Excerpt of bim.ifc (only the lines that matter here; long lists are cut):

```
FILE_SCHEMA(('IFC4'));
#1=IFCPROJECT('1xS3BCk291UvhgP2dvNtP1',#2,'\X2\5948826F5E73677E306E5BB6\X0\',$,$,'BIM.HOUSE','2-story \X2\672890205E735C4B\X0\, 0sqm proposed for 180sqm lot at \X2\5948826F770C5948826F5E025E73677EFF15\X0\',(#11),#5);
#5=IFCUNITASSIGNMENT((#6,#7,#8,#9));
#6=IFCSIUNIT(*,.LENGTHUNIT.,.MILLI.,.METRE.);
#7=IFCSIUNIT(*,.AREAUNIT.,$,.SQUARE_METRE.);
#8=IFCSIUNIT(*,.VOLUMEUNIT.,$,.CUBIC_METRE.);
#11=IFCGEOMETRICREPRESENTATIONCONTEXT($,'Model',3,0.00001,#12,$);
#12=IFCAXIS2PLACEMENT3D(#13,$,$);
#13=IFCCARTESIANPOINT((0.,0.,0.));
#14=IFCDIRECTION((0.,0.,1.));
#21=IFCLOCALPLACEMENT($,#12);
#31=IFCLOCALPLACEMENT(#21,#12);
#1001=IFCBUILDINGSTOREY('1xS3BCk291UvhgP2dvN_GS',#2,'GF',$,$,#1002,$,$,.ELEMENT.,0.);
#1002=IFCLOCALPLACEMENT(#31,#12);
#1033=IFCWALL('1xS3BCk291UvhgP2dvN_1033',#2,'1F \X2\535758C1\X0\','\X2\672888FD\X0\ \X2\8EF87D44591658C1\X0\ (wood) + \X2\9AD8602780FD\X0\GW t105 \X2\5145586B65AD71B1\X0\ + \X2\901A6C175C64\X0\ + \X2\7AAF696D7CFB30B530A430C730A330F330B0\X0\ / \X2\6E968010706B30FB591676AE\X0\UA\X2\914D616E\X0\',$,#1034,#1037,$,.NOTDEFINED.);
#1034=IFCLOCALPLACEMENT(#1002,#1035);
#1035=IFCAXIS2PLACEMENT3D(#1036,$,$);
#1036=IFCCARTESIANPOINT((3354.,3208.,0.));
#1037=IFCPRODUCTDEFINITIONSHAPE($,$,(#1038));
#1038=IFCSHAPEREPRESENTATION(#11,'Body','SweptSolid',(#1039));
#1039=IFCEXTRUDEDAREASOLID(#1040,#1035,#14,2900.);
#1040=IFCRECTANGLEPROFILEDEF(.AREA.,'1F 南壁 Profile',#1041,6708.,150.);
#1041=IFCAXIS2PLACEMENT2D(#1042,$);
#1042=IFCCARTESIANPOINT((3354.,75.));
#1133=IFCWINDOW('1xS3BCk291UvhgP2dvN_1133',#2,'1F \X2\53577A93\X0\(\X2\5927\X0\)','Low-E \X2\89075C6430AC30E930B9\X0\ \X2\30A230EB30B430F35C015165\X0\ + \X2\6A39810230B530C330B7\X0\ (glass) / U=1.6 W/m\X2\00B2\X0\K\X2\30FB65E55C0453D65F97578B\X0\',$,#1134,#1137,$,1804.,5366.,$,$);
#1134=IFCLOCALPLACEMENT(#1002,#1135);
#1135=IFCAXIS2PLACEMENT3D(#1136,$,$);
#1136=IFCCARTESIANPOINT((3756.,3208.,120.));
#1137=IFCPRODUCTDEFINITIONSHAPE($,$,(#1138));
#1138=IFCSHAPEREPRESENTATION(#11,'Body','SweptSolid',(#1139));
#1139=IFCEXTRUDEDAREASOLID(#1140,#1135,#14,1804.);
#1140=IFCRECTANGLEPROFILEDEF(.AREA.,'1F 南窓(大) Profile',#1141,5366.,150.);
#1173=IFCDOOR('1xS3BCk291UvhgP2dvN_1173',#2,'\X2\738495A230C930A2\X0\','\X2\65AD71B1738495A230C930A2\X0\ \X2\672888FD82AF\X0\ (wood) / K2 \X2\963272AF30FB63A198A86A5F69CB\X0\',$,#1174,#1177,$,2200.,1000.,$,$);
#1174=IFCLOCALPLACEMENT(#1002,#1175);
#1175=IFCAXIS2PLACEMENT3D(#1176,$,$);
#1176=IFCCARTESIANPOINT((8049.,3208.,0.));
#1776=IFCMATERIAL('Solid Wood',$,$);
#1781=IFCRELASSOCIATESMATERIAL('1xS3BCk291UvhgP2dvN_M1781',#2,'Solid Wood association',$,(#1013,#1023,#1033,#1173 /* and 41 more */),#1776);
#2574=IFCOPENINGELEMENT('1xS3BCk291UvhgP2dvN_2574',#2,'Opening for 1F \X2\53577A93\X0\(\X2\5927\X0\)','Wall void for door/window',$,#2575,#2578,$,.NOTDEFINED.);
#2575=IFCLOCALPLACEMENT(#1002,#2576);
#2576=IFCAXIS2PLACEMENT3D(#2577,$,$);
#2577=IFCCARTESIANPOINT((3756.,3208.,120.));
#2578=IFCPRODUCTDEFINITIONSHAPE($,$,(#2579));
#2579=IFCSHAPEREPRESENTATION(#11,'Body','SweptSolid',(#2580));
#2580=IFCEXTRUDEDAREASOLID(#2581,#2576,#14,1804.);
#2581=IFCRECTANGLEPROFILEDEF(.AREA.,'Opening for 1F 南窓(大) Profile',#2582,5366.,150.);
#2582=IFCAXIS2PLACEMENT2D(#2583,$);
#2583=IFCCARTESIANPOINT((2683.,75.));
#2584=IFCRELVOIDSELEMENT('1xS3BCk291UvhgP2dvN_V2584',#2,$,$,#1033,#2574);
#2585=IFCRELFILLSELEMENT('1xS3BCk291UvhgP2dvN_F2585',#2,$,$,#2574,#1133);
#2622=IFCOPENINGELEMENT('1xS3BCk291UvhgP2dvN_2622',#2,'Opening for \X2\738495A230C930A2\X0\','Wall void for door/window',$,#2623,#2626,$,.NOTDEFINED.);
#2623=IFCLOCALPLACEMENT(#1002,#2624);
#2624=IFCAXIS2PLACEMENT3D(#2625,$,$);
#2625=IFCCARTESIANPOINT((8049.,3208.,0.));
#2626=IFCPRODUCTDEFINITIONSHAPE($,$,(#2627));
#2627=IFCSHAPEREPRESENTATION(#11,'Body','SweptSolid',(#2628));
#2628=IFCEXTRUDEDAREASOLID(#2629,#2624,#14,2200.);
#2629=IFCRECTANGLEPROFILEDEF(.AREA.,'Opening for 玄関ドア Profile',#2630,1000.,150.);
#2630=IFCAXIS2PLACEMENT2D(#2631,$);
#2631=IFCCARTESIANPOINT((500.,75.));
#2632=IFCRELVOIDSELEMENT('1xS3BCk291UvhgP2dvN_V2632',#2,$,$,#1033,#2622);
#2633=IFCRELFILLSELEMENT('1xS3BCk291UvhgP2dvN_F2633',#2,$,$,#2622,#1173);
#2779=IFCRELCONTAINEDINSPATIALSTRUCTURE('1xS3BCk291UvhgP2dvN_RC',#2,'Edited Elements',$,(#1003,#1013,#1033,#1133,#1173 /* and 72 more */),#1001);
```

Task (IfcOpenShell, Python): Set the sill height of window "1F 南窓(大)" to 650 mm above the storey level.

```python
import numpy as np
import ifcopenshell
import ifcopenshell.api.geometry
import ifcopenshell.geom
import ifcopenshell.util.element
import ifcopenshell.util.placement
import ifcopenshell.util.shape
import ifcopenshell.util.unit

model = ifcopenshell.open("bim.ifc")
unit_scale = ifcopenshell.util.unit.calculate_unit_scale(model)

window = model.by_guid("1xS3BCk291UvhgP2dvN_1133")
opening = window.FillsVoids[0].RelatingOpeningElement
storey = ifcopenshell.util.element.get_container(window, ifc_class="IfcBuildingStorey")
level = ifcopenshell.util.placement.get_local_placement(storey.ObjectPlacement)[2, 3]

# The opening's origin need not be at the sill, so measure its lowest point.
shape = ifcopenshell.geom.create_shape(ifcopenshell.geom.settings(), opening)
bottom = ifcopenshell.util.shape.get_shape_bottom_elevation(shape, shape.geometry) / unit_scale
dz = level + 0.65 / unit_scale - bottom

shift = np.array([0.0, 0.0, dz])
# The window is not placed relative to its opening, so move both.
for product in (opening, window):
    matrix = ifcopenshell.util.placement.get_local_placement(product.ObjectPlacement)
    matrix[:3, 3] += shift
    ifcopenshell.api.geometry.edit_object_placement(model, product=product, matrix=matrix, is_si=False)

print(f"moved by {dz * unit_scale:+.3f} m")

model.write("bim_v2.ifc")
```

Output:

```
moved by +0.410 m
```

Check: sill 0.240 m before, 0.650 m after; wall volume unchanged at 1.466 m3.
